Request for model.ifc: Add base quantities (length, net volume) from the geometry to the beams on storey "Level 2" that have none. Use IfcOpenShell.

First a look at what the model holds.

```python
import ifcopenshell
import ifcopenshell.util.element
import ifcopenshell.util.unit

model = ifcopenshell.open("model.ifc")
print(model.schema)
for unit_type in ("LENGTHUNIT", "AREAUNIT", "VOLUMEUNIT"):
    print(unit_type, ifcopenshell.util.unit.calculate_unit_scale(model, unit_type))
storey = next(s for s in model.by_type("IfcBuildingStorey") if s.Name == "Level 2")
beams = [e for e in ifcopenshell.util.element.get_decomposition(storey) if e.is_a("IfcBeam")]
for e in sorted(beams, key=lambda e: e.id()):
    print(e.id(), e.is_a(), e.Name, list(ifcopenshell.util.element.get_psets(e, qtos_only=True)), sep=" | ")
```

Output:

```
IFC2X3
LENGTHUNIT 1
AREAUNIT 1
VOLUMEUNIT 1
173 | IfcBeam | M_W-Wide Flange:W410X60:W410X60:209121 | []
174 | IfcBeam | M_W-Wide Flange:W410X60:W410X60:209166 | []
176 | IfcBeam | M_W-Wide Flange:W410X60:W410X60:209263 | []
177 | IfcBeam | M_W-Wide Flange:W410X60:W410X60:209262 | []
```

```python
import ifcopenshell
import ifcopenshell.api.pset
import ifcopenshell.geom
import ifcopenshell.util.element
import ifcopenshell.util.shape
import ifcopenshell.util.unit

model = ifcopenshell.open("model.ifc")
unit_scale = ifcopenshell.util.unit.calculate_unit_scale(model)
volume_scale = ifcopenshell.util.unit.calculate_unit_scale(model, "VOLUMEUNIT")
settings = ifcopenshell.geom.settings()

storey = next(s for s in model.by_type("IfcBuildingStorey") if s.Name == "Level 2")
beams = [e for e in ifcopenshell.util.element.get_decomposition(storey) if e.is_a("IfcBeam")]

for e in sorted(beams, key=lambda e: e.id()):
    if ifcopenshell.util.element.get_psets(e, qtos_only=True, should_inherit=False):
        continue
    # Geometry comes back in metres, in the element's own axes.
    shape = ifcopenshell.geom.create_shape(settings, e)
    values = {
        "Length": ifcopenshell.util.shape.get_max_xyz(shape.geometry) / unit_scale,
        "NetVolume": ifcopenshell.util.shape.get_volume(shape.geometry) / volume_scale,
    }
    qto = ifcopenshell.api.pset.add_qto(model, product=e, name="BaseQuantities")
    ifcopenshell.api.pset.edit_qto(model, qto=qto, properties=values)
    print(e.id(), {k: round(v, 3) for k, v in values.items()})

model.write("model_rev.ifc")
```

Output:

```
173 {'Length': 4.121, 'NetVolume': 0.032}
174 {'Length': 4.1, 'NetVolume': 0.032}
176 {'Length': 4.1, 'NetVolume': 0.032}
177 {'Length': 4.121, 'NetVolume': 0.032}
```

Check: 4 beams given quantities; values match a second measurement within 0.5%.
